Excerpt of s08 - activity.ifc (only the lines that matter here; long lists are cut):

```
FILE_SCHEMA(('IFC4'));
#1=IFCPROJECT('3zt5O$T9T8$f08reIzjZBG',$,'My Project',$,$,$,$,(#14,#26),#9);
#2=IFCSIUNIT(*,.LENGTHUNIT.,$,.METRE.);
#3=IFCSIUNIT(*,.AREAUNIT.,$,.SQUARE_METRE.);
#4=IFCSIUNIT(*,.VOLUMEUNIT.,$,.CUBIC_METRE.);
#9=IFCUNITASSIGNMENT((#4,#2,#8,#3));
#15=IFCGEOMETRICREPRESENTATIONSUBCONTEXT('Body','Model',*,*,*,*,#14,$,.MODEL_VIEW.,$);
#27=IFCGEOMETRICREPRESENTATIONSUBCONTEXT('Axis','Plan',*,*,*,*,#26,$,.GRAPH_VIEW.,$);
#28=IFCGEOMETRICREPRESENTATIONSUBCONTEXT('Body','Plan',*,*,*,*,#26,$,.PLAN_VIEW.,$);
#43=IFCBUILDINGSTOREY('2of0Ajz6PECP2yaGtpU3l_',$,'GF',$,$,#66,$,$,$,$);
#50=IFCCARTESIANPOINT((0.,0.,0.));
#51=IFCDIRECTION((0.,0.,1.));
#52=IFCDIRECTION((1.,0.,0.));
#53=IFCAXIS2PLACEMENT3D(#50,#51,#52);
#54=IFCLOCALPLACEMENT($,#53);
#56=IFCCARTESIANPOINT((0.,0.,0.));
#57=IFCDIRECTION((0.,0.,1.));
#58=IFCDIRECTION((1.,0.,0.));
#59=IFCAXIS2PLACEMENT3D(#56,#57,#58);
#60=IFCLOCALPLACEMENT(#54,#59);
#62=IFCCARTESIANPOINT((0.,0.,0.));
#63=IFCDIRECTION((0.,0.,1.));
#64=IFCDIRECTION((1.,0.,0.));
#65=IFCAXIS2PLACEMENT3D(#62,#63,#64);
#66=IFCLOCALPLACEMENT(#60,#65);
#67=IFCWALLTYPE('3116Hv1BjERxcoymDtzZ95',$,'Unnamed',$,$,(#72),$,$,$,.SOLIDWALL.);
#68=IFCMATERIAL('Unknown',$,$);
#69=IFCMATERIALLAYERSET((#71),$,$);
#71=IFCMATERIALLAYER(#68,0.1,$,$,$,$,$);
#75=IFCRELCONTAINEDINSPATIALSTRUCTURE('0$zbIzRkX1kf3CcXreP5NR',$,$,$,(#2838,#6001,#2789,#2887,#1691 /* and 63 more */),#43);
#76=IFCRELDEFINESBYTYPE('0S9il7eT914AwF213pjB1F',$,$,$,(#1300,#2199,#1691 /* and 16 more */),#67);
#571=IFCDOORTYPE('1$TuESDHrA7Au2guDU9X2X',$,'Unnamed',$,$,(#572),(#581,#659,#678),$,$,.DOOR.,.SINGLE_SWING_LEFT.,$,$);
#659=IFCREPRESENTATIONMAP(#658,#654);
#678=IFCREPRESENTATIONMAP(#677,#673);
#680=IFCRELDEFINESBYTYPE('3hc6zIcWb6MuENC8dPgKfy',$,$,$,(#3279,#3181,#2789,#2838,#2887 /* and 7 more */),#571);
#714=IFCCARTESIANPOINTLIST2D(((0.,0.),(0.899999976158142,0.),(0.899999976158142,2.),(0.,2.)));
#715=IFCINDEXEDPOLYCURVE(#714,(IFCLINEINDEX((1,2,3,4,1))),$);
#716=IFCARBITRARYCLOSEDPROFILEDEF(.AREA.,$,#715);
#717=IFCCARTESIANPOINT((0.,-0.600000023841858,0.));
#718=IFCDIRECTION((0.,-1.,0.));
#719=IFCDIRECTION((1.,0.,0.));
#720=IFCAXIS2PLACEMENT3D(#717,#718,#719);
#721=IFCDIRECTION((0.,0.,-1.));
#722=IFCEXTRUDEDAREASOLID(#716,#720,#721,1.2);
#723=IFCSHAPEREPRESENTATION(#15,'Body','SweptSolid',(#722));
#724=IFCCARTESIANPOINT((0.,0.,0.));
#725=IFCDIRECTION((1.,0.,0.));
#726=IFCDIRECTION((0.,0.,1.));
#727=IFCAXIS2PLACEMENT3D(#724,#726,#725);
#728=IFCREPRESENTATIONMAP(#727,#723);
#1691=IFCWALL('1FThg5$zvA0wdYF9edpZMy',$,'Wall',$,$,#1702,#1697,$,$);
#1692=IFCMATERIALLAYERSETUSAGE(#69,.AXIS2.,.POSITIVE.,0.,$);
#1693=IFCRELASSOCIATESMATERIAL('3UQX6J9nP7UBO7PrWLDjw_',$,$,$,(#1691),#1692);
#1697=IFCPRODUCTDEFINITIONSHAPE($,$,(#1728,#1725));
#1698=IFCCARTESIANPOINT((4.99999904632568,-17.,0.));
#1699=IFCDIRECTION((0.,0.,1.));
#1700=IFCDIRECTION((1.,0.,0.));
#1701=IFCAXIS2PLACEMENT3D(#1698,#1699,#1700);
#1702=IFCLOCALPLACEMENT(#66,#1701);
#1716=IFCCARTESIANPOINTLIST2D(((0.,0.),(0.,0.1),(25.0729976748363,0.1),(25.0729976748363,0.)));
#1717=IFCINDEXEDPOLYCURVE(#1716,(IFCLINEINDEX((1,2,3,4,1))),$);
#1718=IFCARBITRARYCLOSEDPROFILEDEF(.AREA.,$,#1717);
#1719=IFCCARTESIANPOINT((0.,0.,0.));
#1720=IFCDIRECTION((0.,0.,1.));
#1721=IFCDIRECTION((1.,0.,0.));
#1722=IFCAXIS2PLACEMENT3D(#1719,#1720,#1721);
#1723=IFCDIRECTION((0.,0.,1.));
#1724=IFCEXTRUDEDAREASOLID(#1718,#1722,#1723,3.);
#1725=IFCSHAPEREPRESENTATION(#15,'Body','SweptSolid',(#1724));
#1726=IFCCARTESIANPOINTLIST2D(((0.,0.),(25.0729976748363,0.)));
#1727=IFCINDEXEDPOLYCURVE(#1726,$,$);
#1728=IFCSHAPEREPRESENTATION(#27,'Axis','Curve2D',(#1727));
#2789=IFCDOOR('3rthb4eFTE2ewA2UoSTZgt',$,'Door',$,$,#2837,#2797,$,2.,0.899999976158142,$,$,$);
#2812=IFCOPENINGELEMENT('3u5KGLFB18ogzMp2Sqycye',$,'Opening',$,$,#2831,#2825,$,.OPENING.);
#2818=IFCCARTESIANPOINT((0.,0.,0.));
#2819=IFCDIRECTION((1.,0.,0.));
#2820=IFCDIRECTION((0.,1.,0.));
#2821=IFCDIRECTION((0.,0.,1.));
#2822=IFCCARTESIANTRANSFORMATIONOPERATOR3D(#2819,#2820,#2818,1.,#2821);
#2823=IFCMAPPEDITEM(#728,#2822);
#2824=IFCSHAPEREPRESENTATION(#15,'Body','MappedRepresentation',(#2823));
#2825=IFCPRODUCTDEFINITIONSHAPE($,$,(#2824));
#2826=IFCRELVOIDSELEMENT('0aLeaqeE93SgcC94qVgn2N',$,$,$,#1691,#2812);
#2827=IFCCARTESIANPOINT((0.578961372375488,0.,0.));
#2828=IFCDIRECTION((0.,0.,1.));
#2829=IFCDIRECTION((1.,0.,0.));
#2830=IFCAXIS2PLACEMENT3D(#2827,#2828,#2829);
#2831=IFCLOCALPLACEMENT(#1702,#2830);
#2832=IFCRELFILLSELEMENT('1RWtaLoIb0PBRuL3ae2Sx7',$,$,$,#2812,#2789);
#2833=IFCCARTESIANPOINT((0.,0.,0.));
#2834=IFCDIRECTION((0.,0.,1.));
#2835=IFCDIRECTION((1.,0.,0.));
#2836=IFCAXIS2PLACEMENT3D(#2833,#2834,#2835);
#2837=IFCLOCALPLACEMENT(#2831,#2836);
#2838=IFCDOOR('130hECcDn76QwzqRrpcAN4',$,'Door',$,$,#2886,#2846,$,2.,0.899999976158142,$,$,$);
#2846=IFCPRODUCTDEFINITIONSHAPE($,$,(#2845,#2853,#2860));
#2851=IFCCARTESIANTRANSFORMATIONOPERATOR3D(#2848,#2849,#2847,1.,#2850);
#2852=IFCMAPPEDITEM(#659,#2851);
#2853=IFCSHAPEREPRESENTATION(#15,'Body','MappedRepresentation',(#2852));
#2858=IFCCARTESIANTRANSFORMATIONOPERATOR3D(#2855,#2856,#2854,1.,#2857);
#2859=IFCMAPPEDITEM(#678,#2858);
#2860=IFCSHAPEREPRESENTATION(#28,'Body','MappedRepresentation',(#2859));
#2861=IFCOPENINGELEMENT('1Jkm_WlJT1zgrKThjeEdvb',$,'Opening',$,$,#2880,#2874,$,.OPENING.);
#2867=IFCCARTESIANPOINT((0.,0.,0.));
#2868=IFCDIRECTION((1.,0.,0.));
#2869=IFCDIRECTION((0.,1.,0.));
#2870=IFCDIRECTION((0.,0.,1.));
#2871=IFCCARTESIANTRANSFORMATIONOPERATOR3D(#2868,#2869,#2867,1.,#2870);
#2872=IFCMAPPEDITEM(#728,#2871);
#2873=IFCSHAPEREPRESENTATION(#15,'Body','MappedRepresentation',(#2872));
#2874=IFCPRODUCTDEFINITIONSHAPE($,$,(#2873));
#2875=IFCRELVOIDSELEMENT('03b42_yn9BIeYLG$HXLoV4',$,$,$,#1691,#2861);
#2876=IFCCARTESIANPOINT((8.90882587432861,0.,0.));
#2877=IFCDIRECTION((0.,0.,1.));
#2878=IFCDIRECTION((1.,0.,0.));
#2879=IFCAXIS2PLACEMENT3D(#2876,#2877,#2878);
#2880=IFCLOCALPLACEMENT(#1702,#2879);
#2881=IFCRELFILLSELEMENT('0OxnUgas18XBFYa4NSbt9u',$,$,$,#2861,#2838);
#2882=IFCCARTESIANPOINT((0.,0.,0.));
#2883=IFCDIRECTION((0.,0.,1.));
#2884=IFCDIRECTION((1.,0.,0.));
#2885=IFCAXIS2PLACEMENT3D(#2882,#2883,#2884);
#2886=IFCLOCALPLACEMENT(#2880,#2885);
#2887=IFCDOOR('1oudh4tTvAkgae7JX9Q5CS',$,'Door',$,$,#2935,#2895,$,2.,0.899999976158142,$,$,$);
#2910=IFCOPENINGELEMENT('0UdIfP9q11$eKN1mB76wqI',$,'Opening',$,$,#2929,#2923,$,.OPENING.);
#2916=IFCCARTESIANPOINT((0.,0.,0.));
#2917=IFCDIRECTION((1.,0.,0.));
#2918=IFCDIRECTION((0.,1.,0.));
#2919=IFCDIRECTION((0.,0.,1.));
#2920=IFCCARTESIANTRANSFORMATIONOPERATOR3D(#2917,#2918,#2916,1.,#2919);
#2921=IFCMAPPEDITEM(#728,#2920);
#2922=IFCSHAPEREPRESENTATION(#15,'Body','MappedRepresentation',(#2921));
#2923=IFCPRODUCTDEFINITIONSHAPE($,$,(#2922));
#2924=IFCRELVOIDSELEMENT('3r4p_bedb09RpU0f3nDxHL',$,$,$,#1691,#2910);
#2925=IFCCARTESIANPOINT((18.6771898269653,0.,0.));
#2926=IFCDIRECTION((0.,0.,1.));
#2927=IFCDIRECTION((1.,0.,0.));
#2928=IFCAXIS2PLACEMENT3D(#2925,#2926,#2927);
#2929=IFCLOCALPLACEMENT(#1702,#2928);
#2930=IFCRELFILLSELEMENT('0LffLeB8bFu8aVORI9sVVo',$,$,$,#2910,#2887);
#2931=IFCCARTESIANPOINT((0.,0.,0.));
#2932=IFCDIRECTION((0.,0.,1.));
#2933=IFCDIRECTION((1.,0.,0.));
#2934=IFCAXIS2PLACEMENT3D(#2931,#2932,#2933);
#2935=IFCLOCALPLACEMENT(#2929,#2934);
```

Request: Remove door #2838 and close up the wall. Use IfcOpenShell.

```python
import ifcopenshell
import ifcopenshell.api.feature
import ifcopenshell.api.root
import ifcopenshell.geom
import ifcopenshell.util.shape

model = ifcopenshell.open("s08 - activity.ifc")
settings = ifcopenshell.geom.settings()


def volume(element):
    """Net volume in cubic metres, openings subtracted."""
    shape = ifcopenshell.geom.create_shape(settings, element)
    return ifcopenshell.util.shape.get_volume(shape.geometry)


door = model.by_id(2838)
opening = door.FillsVoids[0].RelatingOpeningElement
wall = opening.VoidsElements[0].RelatingBuildingElement
before = volume(wall)

ifcopenshell.api.root.remove_product(model, product=door)
ifcopenshell.api.feature.remove_feature(model, feature=opening)

after = volume(wall)

print(f"wall volume {before:.3f} -> {after:.3f} m3")

model.write("s08 - activity_updated.ifc")
```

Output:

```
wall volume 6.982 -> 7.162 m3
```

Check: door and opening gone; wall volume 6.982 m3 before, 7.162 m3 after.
